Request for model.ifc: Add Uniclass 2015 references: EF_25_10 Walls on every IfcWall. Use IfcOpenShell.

First a look at what the model holds.

```python
import ifcopenshell

model = ifcopenshell.open("model.ifc")
print(model.schema)
print("classifications:", [c.Name for c in model.by_type("IfcClassification")])
for ifc_class in ("IfcDoor", "IfcRoof", "IfcStair", "IfcWall", "IfcWindow"):
    print(ifc_class, len(model.by_type(ifc_class)))
```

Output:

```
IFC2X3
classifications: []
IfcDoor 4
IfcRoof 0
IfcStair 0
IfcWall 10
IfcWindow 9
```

```python
import ifcopenshell
import ifcopenshell.api.classification

model = ifcopenshell.open("model.ifc")

# IFC2X3 requires Source and Edition and has no link from the project to the system.
system = model.create_entity("IfcClassification", Source="NBS", Edition="2015", Name="Uniclass 2015")

codes = {
    "IfcWall": ("EF_25_10", "Walls"),
}
for ifc_class, (code, name) in codes.items():
    products = model.by_type(ifc_class)
    ifcopenshell.api.classification.add_reference(
        model, products=products, classification=system, identification=code, name=name
    )
    print(code, len(products))

model.write("model_rev.ifc")
```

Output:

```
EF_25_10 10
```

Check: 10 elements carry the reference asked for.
